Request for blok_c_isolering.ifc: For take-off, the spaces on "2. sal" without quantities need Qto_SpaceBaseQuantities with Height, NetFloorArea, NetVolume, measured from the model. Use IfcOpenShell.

First a look at what the model holds.

```python
import ifcopenshell
import ifcopenshell.util.element
import ifcopenshell.util.unit

model = ifcopenshell.open("blok_c_isolering.ifc")
print(model.schema)
for unit_type in ("LENGTHUNIT", "AREAUNIT", "VOLUMEUNIT"):
    print(unit_type, ifcopenshell.util.unit.calculate_unit_scale(model, unit_type))
storey = next(s for s in model.by_type("IfcBuildingStorey") if s.Name == "2. sal")
spaces = [e for e in ifcopenshell.util.element.get_decomposition(storey) if e.is_a("IfcSpace")]
for e in sorted(spaces, key=lambda e: e.id()):
    print(e.id(), e.is_a(), e.Name, list(ifcopenshell.util.element.get_psets(e, qtos_only=True)), sep=" | ")
```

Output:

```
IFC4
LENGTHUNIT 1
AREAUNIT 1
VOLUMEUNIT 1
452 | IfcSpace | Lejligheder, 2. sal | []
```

```python
import ifcopenshell
import ifcopenshell.api.pset
import ifcopenshell.geom
import ifcopenshell.util.element
import ifcopenshell.util.shape
import ifcopenshell.util.unit

model = ifcopenshell.open("blok_c_isolering.ifc")
unit_scale = ifcopenshell.util.unit.calculate_unit_scale(model)
area_scale = ifcopenshell.util.unit.calculate_unit_scale(model, "AREAUNIT")
volume_scale = ifcopenshell.util.unit.calculate_unit_scale(model, "VOLUMEUNIT")
settings = ifcopenshell.geom.settings()

storey = next(s for s in model.by_type("IfcBuildingStorey") if s.Name == "2. sal")
spaces = [e for e in ifcopenshell.util.element.get_decomposition(storey) if e.is_a("IfcSpace")]

for e in sorted(spaces, key=lambda e: e.id()):
    if ifcopenshell.util.element.get_psets(e, qtos_only=True, should_inherit=False):
        continue
    # Geometry comes back in metres, in the element's own axes.
    shape = ifcopenshell.geom.create_shape(settings, e)
    values = {
        "Height": ifcopenshell.util.shape.get_z(shape.geometry) / unit_scale,
        "NetFloorArea": ifcopenshell.util.shape.get_footprint_area(shape.geometry) / area_scale,
        "NetVolume": ifcopenshell.util.shape.get_volume(shape.geometry) / volume_scale,
    }
    qto = ifcopenshell.api.pset.add_qto(model, product=e, name="Qto_SpaceBaseQuantities")
    ifcopenshell.api.pset.edit_qto(model, qto=qto, properties=values)
    print(e.id(), {k: round(v, 3) for k, v in values.items()})

model.write("blok_c_isolering_updated.ifc")
```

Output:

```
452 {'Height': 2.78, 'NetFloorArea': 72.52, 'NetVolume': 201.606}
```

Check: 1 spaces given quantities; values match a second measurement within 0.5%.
